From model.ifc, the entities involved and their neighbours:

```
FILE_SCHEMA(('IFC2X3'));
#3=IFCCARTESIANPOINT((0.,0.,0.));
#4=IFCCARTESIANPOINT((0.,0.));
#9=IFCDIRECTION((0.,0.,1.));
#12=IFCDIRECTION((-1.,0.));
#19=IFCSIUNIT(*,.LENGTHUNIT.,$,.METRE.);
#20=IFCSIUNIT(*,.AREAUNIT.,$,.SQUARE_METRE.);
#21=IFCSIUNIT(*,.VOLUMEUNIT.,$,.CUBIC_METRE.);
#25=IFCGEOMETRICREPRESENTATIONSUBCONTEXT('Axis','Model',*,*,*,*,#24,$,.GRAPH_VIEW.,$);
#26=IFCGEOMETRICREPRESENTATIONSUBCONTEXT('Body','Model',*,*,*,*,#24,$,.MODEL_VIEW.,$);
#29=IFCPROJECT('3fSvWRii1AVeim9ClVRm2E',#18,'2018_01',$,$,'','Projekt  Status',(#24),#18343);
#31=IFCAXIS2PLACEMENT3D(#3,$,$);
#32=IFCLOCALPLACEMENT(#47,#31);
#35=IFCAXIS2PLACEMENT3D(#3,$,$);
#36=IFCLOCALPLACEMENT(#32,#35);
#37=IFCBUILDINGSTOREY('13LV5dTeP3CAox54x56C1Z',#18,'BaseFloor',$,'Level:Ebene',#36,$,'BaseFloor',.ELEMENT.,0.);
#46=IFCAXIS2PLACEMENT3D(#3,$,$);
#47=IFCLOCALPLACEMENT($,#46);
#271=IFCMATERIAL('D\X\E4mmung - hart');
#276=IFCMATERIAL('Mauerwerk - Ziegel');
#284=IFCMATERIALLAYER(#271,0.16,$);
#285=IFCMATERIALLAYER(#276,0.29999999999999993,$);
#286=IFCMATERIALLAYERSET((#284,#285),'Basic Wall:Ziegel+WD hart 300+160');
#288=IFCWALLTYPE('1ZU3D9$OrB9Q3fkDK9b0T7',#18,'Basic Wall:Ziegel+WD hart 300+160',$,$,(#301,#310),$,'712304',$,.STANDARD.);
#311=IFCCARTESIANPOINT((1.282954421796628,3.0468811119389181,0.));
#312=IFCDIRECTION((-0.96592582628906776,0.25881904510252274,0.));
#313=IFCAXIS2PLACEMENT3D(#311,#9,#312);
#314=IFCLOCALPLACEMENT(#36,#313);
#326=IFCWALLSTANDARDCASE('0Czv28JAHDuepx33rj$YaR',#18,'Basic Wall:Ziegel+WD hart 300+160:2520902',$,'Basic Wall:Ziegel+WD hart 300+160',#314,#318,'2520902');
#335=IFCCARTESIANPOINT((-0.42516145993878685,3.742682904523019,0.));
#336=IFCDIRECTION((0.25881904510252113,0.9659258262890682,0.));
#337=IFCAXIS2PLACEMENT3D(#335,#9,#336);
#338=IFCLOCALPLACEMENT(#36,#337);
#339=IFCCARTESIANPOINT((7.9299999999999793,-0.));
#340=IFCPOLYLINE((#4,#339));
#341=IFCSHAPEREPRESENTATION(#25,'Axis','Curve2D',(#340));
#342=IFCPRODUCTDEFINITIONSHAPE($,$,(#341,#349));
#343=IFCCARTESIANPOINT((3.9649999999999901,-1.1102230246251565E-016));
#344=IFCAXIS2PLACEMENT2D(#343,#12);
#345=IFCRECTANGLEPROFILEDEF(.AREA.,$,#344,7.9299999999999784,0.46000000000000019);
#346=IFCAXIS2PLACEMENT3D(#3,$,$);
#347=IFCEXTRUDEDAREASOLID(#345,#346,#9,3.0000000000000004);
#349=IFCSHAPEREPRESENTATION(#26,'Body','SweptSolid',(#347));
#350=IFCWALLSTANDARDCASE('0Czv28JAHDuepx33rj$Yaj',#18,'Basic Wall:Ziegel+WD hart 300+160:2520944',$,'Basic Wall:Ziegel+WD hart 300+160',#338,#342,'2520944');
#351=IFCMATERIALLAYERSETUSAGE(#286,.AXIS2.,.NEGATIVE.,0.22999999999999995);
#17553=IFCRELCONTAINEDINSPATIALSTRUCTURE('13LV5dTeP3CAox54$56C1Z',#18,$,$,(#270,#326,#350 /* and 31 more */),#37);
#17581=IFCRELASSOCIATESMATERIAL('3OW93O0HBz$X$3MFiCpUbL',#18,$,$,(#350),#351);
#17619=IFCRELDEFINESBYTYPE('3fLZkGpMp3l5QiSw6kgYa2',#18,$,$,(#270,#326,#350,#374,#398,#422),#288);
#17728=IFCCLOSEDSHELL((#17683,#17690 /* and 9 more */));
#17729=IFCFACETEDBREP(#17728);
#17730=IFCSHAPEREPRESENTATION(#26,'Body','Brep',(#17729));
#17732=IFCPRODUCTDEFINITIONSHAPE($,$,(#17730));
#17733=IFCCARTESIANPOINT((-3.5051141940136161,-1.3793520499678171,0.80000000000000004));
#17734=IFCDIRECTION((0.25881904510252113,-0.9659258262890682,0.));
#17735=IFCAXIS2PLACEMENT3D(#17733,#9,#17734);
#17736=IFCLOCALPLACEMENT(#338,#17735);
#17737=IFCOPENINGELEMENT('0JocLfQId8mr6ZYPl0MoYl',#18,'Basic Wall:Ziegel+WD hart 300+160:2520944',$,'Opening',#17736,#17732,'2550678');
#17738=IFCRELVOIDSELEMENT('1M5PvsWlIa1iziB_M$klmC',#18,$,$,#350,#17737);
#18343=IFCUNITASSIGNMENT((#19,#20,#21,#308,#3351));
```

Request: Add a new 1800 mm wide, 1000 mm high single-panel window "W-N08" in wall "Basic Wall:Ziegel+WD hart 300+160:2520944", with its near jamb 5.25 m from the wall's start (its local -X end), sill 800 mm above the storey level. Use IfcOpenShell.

```python
import numpy as np
import ifcopenshell
import ifcopenshell.api.feature
import ifcopenshell.api.geometry
import ifcopenshell.api.root
import ifcopenshell.api.spatial
import ifcopenshell.api.type
import ifcopenshell.geom
import ifcopenshell.util.element
import ifcopenshell.util.placement
import ifcopenshell.util.representation
import ifcopenshell.util.shape
import ifcopenshell.util.unit

model = ifcopenshell.open("model.ifc")
unit_scale = ifcopenshell.util.unit.calculate_unit_scale(model)
settings = ifcopenshell.geom.settings()


def volume(element):
    """Net volume in cubic metres, openings subtracted."""
    shape = ifcopenshell.geom.create_shape(settings, element)
    return ifcopenshell.util.shape.get_volume(shape.geometry)


wall = model.by_guid("0Czv28JAHDuepx33rj$Yaj")
storey = ifcopenshell.util.element.get_container(wall, ifc_class="IfcBuildingStorey")
context = ifcopenshell.util.representation.get_context(model, "Model", "Body", "MODEL_VIEW")
before = volume(wall)

width, height, from_end, sill = 1.8, 1, 5.25, 0.8  # metres

# The wall runs along its own X axis, and the end named is its -X end.
wall_shape = ifcopenshell.geom.create_shape(settings, wall)
x, y, z = ifcopenshell.util.shape.get_vertices(wall_shape.geometry).T
start = x.min() + from_end
face, thickness = float(y.min()), float(y.max() - y.min())
wall_matrix = ifcopenshell.util.placement.get_local_placement(wall.ObjectPlacement)
level = ifcopenshell.util.placement.get_local_placement(storey.ObjectPlacement)[2, 3]


def in_wall(x, y):
    """Placement at x, y metres in the wall's axes, at sill height."""
    matrix = wall_matrix.copy()
    matrix[:, 3] = wall_matrix @ np.array([x / unit_scale, y / unit_scale, 0.0, 1.0])
    matrix[2, 3] = level + sill / unit_scale
    return matrix


# Opening: a box that overshoots both wall faces by 50 mm.
opening = ifcopenshell.api.root.create_entity(model, ifc_class="IfcOpeningElement")
box = ifcopenshell.api.geometry.add_wall_representation(
    model, context=context, length=width, height=height, thickness=thickness + 0.1
)
ifcopenshell.api.geometry.assign_representation(model, product=opening, representation=box)
ifcopenshell.api.geometry.edit_object_placement(model, product=opening, matrix=in_wall(start, face - 0.05), is_si=False)
ifcopenshell.api.feature.add_feature(model, feature=opening, element=wall)

window = ifcopenshell.api.root.create_entity(model, ifc_class="IfcWindow", name="W-N08")
window.OverallWidth, window.OverallHeight = width / unit_scale, height / unit_scale
body = ifcopenshell.api.geometry.add_window_representation(
    model,
    context=context,
    overall_width=window.OverallWidth,
    overall_height=window.OverallHeight,
    partition_type="SINGLE_PANEL",
)
ifcopenshell.api.geometry.assign_representation(model, product=window, representation=body)
ifcopenshell.api.spatial.assign_container(model, products=[window], relating_structure=storey)
fills = ifcopenshell.api.feature.add_filling(model, opening=opening, element=window)
fills.OwnerHistory = window.OwnerHistory  # required in IFC2X3

# IFC2X3 keeps the operation on the window style.
style = ifcopenshell.api.root.create_entity(model, ifc_class="IfcWindowStyle", name="W-N08")
style.OperationType, style.ConstructionType = "SINGLE_PANEL", "NOTDEFINED"
style.ParameterTakesPrecedence = style.Sizeable = False
ifcopenshell.api.type.assign_type(model, related_objects=[window], relating_type=style)

# Centre the window in the wall's thickness.
ifcopenshell.api.geometry.edit_object_placement(model, product=window, matrix=in_wall(start, face), is_si=False)
window_shape = ifcopenshell.geom.create_shape(settings, window)
depth = ifcopenshell.util.shape.get_vertices(window_shape.geometry)[:, 1]
offset = face + thickness / 2 - (depth.min() + depth.max()) / 2
ifcopenshell.api.geometry.edit_object_placement(model, product=window, matrix=in_wall(start, offset), is_si=False)

after = volume(wall)

print(f"wall volume {before:.3f} -> {after:.3f} m3")

model.write("model_updated.ifc")
```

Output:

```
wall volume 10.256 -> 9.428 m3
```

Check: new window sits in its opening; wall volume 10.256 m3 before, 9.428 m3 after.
